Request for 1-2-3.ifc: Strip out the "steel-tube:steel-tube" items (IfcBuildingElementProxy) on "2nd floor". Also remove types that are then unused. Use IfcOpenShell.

First a look at what the model holds.

```python
import ifcopenshell
import ifcopenshell.util.element

model = ifcopenshell.open("1-2-3.ifc")
print(model.schema)
storey = next(s for s in model.by_type("IfcBuildingStorey") if s.Name == "2nd floor")
proxies = [e for e in ifcopenshell.util.element.get_decomposition(storey) if e.is_a("IfcBuildingElementProxy")]
seen = {}
for e in proxies:
    element_type = ifcopenshell.util.element.get_type(e)
    name = element_type.Name if element_type not in (None, e) else None
    seen[name] = seen.get(name, 0) + 1
for name, count in sorted(seen.items(), key=str):
    print(count, "x", name)
```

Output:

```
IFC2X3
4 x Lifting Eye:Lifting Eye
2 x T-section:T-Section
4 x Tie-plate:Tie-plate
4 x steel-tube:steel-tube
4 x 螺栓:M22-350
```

```python
import ifcopenshell
import ifcopenshell.api.root
import ifcopenshell.util.element

model = ifcopenshell.open("1-2-3.ifc")

storey = next(s for s in model.by_type("IfcBuildingStorey") if s.Name == "2nd floor")
proxies = [e for e in ifcopenshell.util.element.get_decomposition(storey) if e.is_a("IfcBuildingElementProxy")]
targets = [e for e in proxies if (t := ifcopenshell.util.element.get_type(e)) not in (None, e) and t.Name == "steel-tube:steel-tube"]
types = {ifcopenshell.util.element.get_type(e) for e in targets} - {None, *targets}

for e in targets:
    ifcopenshell.api.root.remove_product(model, product=e)
print(len(targets), "removed")

unused = [t for t in types if not ifcopenshell.util.element.get_types(t)]
for t in unused:
    ifcopenshell.api.root.remove_product(model, product=t)
print(len(unused), "unused types removed")

model.write("1-2-3_v2.ifc")
```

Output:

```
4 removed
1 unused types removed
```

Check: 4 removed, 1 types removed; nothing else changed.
